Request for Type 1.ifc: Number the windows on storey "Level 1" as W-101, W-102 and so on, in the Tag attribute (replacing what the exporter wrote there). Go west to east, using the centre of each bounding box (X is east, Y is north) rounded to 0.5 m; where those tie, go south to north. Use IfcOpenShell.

First a look at what the model holds.

```python
import ifcopenshell
import ifcopenshell.util.element
import ifcopenshell.util.placement

model = ifcopenshell.open("Type 1.ifc")
print(model.schema)
storey = next(s for s in model.by_type("IfcBuildingStorey") if s.Name == "Level 1")
windows = [e for e in ifcopenshell.util.element.get_decomposition(storey) if e.is_a("IfcWindow")]
for e in sorted(windows, key=lambda e: e.id()):
    origin = ifcopenshell.util.placement.get_local_placement(e.ObjectPlacement)[:3, 3]
    print(e.id(), e.Tag, e.Name, origin.round(2) + 0.0, sep=" | ")
```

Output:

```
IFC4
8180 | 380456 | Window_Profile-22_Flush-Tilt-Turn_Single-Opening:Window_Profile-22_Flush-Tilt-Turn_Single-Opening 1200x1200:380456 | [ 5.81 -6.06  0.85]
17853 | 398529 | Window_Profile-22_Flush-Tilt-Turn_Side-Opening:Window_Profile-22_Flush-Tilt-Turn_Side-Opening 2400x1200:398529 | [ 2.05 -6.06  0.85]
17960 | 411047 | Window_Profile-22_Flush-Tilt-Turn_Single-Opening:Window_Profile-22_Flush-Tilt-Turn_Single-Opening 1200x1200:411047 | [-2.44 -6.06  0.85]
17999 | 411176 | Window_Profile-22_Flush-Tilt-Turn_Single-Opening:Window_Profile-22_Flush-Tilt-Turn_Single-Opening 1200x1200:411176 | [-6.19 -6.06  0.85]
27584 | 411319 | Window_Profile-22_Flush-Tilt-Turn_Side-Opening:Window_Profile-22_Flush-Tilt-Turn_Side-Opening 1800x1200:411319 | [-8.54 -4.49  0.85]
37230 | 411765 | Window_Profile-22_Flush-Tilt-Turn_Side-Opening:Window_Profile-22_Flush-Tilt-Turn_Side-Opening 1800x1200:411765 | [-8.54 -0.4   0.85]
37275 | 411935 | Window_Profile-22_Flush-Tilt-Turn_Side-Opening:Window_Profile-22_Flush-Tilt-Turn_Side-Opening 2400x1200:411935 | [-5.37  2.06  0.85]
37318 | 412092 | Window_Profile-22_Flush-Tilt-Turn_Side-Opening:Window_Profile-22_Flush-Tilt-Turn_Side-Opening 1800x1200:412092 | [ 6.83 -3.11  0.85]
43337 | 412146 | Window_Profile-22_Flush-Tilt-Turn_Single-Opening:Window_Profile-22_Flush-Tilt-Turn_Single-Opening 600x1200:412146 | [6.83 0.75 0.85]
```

```python
import ifcopenshell
import ifcopenshell.geom
import ifcopenshell.util.element
import ifcopenshell.util.shape

model = ifcopenshell.open("Type 1.ifc")
settings = ifcopenshell.geom.settings()
settings.set("use-world-coords", True)


def centre(element):
    shape = ifcopenshell.geom.create_shape(settings, element)
    return ifcopenshell.util.shape.get_bbox_centroid(shape.geometry)


storey = next(s for s in model.by_type("IfcBuildingStorey") if s.Name == "Level 1")
windows = [e for e in ifcopenshell.util.element.get_decomposition(storey) if e.is_a("IfcWindow")]

# Insertion points can sit at a corner or the storey origin, so sort by the geometry (in metres).
centres = {e: centre(e) for e in windows}
windows.sort(key=lambda e: (round(centres[e][0] / 0.5), centres[e][1]))

for i, e in enumerate(windows, start=1):
    number = f"W-1{i:02d}"
    e.Tag = number
    print(e.id(), number)

model.write("Type 1_v2.ifc")
```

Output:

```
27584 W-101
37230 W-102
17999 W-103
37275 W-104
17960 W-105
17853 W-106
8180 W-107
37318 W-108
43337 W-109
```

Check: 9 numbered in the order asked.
